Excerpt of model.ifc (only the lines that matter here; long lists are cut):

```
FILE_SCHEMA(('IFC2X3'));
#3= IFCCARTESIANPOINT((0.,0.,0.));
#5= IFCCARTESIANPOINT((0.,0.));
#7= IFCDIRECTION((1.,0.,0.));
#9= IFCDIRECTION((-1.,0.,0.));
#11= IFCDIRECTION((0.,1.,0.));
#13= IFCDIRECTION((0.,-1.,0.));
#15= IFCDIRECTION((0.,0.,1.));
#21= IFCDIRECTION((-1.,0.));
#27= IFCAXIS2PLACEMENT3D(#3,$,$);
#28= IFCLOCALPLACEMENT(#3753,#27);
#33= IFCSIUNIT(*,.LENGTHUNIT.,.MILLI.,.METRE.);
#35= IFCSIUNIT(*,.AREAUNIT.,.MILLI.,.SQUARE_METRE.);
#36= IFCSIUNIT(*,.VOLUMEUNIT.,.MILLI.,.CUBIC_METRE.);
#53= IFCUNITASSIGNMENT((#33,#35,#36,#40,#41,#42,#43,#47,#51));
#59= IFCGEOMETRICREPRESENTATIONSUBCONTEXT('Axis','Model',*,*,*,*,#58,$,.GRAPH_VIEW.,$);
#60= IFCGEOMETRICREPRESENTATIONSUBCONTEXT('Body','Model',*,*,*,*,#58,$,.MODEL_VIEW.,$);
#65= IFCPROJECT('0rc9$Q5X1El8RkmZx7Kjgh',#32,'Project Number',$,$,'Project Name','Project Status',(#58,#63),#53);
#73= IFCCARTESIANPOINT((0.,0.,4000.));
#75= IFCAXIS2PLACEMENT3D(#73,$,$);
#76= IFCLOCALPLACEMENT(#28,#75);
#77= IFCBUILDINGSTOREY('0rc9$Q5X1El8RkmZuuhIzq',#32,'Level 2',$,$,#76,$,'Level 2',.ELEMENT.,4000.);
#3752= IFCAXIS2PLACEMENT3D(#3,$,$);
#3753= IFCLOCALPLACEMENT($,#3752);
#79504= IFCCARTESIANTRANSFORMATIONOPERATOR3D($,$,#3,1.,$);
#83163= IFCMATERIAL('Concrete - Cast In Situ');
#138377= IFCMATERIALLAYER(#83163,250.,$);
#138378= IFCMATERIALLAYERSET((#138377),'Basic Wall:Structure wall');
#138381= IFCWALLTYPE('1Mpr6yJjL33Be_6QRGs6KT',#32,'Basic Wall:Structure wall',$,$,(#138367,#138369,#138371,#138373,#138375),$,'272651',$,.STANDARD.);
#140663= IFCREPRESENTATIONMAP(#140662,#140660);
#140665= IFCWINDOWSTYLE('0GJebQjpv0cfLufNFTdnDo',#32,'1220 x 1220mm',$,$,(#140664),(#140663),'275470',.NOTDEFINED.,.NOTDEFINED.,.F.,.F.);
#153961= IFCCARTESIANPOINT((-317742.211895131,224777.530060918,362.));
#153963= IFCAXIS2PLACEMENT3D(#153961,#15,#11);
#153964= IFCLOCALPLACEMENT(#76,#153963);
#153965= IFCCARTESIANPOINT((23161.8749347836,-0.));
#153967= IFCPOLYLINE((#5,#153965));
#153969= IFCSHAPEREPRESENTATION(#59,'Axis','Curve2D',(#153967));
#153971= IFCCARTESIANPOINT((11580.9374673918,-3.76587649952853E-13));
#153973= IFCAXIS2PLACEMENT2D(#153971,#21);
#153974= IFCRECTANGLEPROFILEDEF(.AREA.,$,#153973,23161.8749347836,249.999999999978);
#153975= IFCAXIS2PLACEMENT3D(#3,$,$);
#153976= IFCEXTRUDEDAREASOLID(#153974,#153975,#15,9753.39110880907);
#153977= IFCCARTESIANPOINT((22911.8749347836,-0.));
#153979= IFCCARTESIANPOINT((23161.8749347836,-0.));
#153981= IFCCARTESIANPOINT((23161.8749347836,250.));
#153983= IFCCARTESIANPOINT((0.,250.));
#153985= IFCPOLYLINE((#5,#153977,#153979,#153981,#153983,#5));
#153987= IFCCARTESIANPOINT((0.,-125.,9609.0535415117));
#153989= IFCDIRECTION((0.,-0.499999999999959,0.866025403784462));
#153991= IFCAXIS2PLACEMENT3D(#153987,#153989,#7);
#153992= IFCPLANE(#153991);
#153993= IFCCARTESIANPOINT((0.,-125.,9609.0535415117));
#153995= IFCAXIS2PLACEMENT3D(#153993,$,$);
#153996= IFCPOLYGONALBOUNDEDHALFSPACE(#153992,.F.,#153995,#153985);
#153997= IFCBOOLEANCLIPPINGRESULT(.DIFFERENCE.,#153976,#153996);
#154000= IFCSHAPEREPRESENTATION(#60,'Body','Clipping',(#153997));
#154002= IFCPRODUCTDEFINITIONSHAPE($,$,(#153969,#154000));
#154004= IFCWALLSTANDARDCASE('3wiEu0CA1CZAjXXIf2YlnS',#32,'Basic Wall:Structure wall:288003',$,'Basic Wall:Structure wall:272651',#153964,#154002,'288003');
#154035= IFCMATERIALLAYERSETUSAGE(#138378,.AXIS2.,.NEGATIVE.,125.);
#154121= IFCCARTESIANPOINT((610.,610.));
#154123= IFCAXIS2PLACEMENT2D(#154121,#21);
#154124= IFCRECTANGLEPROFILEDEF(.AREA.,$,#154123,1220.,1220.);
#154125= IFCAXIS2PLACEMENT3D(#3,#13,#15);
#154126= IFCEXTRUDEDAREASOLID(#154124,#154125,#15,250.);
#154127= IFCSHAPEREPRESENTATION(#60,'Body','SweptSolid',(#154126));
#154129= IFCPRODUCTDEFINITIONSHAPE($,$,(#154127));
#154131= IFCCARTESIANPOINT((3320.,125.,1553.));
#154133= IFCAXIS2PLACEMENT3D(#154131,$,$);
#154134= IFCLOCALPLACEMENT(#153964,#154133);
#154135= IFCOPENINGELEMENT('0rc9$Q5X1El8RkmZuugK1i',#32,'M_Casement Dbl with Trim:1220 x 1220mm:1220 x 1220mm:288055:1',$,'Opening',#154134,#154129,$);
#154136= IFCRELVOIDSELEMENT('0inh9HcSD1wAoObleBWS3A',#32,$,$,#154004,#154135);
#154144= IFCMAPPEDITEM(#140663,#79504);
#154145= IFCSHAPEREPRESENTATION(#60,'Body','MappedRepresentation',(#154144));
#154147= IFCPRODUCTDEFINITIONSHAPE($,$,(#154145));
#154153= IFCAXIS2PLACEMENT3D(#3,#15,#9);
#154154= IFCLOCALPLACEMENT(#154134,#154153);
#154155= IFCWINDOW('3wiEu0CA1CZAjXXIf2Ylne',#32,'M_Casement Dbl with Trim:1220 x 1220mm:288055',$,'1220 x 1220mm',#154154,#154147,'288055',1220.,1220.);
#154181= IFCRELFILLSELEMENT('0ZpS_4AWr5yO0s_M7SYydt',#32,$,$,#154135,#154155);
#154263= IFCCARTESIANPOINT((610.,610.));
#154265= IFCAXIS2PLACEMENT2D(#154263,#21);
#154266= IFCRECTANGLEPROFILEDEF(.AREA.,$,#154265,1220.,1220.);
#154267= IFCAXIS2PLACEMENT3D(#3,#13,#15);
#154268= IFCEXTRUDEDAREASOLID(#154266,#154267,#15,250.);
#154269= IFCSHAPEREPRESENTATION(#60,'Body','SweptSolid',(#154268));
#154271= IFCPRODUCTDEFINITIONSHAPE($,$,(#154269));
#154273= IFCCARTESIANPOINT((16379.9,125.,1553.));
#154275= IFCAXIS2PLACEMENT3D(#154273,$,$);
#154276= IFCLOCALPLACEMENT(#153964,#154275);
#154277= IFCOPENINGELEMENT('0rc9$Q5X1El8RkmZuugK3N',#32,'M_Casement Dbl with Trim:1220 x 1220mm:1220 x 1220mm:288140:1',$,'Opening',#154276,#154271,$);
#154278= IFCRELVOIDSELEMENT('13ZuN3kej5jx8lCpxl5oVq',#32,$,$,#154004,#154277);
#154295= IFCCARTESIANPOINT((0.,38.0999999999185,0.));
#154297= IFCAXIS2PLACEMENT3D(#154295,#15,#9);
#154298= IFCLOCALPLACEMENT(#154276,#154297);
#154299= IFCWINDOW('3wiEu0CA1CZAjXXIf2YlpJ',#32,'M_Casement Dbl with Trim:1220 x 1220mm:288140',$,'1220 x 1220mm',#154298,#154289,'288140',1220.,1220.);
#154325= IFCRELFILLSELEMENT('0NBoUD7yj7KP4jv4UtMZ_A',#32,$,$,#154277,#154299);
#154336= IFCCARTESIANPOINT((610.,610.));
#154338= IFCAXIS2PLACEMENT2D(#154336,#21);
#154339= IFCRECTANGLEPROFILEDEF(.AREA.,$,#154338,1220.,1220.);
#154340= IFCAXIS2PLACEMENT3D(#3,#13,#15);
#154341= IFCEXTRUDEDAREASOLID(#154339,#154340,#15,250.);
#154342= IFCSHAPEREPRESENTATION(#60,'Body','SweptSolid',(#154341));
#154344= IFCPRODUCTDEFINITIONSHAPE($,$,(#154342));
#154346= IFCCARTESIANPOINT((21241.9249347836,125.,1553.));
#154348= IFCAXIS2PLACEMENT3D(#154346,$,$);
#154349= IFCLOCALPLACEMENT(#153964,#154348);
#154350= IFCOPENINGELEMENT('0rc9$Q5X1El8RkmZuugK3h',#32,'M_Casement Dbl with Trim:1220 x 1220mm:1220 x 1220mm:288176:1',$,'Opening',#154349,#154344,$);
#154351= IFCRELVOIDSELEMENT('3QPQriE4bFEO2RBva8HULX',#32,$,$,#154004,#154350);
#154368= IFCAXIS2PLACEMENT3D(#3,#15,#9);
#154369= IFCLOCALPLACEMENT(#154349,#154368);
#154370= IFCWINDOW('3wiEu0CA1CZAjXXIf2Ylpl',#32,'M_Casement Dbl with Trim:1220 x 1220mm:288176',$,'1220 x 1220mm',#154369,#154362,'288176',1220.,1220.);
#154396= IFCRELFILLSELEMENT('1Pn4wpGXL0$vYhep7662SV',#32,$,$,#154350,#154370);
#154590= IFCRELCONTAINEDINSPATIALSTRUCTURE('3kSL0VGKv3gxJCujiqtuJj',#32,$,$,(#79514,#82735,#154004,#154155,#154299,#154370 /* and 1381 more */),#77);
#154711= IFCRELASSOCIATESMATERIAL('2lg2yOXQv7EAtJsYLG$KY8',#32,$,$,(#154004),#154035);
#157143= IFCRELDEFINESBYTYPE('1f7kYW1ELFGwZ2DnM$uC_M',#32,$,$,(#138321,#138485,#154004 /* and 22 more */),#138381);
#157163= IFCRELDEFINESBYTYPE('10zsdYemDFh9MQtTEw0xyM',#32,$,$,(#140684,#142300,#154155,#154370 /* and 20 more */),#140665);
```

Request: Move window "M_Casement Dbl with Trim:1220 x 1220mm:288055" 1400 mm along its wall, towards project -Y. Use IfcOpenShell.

```python
import ifcopenshell
import ifcopenshell.api.geometry
import ifcopenshell.util.placement

model = ifcopenshell.open("model.ifc")

window = model.by_guid("3wiEu0CA1CZAjXXIf2Ylne")
opening = window.FillsVoids[0].RelatingOpeningElement
wall = opening.VoidsElements[0].RelatingBuildingElement

wall_matrix = ifcopenshell.util.placement.get_local_placement(wall.ObjectPlacement)
shift = wall_matrix[:3, 0] * -1400.0
before = ifcopenshell.util.placement.get_local_placement(window.ObjectPlacement)[:3, 3].copy()

# The window is placed relative to its opening, so it follows when the opening moves.
matrix = ifcopenshell.util.placement.get_local_placement(opening.ObjectPlacement)
matrix[:3, 3] += shift
ifcopenshell.api.geometry.edit_object_placement(
    model, product=opening, matrix=matrix, is_si=False, should_transform_children=True
)

after = ifcopenshell.util.placement.get_local_placement(window.ObjectPlacement)[:3, 3]
print("window moved by", (after - before).round(3) + 0.0)

model.write("model_updated.ifc")
```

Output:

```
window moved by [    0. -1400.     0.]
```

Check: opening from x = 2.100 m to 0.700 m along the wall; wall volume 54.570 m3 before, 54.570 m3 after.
